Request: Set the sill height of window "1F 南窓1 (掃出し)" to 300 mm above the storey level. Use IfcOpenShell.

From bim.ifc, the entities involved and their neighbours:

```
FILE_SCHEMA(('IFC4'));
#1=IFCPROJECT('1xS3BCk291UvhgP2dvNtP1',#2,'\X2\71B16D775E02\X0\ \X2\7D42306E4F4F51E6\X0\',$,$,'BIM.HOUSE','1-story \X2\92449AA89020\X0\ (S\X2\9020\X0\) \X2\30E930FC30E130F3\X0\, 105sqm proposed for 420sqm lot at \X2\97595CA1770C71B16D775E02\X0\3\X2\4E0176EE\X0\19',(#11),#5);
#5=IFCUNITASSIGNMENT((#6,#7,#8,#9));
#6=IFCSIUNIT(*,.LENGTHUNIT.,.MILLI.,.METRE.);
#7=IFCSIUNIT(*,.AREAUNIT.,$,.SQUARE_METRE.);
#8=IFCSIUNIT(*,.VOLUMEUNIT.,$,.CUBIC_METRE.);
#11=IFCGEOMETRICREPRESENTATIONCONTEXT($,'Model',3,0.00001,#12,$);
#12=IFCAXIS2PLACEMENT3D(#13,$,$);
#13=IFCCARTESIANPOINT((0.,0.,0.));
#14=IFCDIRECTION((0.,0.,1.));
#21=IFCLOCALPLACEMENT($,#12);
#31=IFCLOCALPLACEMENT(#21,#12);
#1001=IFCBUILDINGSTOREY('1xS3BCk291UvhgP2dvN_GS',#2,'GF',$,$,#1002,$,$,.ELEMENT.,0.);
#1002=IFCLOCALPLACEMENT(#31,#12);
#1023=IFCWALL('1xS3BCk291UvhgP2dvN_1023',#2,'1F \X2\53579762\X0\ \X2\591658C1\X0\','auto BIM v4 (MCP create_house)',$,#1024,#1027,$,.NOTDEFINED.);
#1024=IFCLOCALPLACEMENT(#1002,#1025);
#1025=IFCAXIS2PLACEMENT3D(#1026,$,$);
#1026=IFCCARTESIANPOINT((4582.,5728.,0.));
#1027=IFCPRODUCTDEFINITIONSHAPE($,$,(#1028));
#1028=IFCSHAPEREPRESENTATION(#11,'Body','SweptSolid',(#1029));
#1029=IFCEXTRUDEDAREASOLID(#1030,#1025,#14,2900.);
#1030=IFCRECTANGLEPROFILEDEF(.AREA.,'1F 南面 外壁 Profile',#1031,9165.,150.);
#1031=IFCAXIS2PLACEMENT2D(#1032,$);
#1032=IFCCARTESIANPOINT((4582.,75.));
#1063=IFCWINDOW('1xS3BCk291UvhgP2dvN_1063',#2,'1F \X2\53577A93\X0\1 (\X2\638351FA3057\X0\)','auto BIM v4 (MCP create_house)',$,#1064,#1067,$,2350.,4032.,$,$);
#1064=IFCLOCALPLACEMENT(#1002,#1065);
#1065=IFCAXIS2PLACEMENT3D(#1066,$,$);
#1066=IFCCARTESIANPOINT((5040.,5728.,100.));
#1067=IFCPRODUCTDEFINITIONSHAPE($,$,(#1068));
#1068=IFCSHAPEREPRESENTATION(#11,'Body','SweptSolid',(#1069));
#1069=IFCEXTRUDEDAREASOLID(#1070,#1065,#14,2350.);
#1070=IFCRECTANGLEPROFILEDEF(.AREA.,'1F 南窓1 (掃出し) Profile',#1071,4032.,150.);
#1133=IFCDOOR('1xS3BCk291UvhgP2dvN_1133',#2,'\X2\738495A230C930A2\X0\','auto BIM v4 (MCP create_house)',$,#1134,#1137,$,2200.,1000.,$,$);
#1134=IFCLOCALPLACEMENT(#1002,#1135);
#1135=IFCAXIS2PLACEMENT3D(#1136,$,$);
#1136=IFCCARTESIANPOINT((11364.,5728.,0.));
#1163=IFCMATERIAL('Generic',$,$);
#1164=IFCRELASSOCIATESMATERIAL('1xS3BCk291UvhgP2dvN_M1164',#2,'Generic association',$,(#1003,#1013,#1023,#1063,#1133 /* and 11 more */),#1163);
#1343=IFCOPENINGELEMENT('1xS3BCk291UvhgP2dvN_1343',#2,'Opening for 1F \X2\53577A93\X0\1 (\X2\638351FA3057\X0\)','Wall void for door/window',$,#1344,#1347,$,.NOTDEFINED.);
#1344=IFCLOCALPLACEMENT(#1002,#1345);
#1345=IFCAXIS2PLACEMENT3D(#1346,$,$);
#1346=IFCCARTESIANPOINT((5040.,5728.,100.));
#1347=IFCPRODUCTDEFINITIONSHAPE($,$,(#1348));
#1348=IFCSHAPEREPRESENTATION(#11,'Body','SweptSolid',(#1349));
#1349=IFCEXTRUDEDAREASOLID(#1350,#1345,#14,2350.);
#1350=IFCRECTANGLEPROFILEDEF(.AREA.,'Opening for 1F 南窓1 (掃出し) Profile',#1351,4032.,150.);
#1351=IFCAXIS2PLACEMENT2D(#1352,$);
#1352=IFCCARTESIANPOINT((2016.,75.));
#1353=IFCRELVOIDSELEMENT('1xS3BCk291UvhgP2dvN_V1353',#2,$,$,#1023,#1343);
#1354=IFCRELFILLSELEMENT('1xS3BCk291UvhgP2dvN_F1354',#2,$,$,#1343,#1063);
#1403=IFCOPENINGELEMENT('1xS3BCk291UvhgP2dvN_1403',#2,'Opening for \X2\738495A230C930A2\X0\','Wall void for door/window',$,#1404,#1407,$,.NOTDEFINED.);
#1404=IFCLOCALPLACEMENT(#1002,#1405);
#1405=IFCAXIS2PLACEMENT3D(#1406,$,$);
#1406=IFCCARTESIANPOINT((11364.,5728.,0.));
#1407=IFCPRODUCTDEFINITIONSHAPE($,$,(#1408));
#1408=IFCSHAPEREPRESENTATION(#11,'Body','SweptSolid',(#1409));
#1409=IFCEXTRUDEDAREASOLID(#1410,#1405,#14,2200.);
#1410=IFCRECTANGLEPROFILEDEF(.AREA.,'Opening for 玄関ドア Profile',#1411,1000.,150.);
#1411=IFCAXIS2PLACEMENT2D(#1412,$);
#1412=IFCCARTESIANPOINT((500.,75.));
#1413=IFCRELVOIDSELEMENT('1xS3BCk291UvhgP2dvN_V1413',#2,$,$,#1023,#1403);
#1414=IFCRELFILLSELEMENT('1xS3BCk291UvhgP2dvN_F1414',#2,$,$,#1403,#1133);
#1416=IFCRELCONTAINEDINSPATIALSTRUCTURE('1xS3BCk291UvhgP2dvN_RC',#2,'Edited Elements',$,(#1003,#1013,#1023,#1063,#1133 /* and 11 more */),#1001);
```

```python
import numpy as np
import ifcopenshell
import ifcopenshell.api.geometry
import ifcopenshell.geom
import ifcopenshell.util.element
import ifcopenshell.util.placement
import ifcopenshell.util.shape
import ifcopenshell.util.unit

model = ifcopenshell.open("bim.ifc")
unit_scale = ifcopenshell.util.unit.calculate_unit_scale(model)

window = model.by_guid("1xS3BCk291UvhgP2dvN_1063")
opening = window.FillsVoids[0].RelatingOpeningElement
storey = ifcopenshell.util.element.get_container(window, ifc_class="IfcBuildingStorey")
level = ifcopenshell.util.placement.get_local_placement(storey.ObjectPlacement)[2, 3]

# The opening's origin need not be at the sill, so measure its lowest point.
shape = ifcopenshell.geom.create_shape(ifcopenshell.geom.settings(), opening)
bottom = ifcopenshell.util.shape.get_shape_bottom_elevation(shape, shape.geometry) / unit_scale
dz = level + 0.3 / unit_scale - bottom

shift = np.array([0.0, 0.0, dz])
# The window is not placed relative to its opening, so move both.
for product in (opening, window):
    matrix = ifcopenshell.util.placement.get_local_placement(product.ObjectPlacement)
    matrix[:3, 3] += shift
    ifcopenshell.api.geometry.edit_object_placement(model, product=product, matrix=matrix, is_si=False)

print(f"moved by {dz * unit_scale:+.3f} m")

model.write("bim_v2.ifc")
```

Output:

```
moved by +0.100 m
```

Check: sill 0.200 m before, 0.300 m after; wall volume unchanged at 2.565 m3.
